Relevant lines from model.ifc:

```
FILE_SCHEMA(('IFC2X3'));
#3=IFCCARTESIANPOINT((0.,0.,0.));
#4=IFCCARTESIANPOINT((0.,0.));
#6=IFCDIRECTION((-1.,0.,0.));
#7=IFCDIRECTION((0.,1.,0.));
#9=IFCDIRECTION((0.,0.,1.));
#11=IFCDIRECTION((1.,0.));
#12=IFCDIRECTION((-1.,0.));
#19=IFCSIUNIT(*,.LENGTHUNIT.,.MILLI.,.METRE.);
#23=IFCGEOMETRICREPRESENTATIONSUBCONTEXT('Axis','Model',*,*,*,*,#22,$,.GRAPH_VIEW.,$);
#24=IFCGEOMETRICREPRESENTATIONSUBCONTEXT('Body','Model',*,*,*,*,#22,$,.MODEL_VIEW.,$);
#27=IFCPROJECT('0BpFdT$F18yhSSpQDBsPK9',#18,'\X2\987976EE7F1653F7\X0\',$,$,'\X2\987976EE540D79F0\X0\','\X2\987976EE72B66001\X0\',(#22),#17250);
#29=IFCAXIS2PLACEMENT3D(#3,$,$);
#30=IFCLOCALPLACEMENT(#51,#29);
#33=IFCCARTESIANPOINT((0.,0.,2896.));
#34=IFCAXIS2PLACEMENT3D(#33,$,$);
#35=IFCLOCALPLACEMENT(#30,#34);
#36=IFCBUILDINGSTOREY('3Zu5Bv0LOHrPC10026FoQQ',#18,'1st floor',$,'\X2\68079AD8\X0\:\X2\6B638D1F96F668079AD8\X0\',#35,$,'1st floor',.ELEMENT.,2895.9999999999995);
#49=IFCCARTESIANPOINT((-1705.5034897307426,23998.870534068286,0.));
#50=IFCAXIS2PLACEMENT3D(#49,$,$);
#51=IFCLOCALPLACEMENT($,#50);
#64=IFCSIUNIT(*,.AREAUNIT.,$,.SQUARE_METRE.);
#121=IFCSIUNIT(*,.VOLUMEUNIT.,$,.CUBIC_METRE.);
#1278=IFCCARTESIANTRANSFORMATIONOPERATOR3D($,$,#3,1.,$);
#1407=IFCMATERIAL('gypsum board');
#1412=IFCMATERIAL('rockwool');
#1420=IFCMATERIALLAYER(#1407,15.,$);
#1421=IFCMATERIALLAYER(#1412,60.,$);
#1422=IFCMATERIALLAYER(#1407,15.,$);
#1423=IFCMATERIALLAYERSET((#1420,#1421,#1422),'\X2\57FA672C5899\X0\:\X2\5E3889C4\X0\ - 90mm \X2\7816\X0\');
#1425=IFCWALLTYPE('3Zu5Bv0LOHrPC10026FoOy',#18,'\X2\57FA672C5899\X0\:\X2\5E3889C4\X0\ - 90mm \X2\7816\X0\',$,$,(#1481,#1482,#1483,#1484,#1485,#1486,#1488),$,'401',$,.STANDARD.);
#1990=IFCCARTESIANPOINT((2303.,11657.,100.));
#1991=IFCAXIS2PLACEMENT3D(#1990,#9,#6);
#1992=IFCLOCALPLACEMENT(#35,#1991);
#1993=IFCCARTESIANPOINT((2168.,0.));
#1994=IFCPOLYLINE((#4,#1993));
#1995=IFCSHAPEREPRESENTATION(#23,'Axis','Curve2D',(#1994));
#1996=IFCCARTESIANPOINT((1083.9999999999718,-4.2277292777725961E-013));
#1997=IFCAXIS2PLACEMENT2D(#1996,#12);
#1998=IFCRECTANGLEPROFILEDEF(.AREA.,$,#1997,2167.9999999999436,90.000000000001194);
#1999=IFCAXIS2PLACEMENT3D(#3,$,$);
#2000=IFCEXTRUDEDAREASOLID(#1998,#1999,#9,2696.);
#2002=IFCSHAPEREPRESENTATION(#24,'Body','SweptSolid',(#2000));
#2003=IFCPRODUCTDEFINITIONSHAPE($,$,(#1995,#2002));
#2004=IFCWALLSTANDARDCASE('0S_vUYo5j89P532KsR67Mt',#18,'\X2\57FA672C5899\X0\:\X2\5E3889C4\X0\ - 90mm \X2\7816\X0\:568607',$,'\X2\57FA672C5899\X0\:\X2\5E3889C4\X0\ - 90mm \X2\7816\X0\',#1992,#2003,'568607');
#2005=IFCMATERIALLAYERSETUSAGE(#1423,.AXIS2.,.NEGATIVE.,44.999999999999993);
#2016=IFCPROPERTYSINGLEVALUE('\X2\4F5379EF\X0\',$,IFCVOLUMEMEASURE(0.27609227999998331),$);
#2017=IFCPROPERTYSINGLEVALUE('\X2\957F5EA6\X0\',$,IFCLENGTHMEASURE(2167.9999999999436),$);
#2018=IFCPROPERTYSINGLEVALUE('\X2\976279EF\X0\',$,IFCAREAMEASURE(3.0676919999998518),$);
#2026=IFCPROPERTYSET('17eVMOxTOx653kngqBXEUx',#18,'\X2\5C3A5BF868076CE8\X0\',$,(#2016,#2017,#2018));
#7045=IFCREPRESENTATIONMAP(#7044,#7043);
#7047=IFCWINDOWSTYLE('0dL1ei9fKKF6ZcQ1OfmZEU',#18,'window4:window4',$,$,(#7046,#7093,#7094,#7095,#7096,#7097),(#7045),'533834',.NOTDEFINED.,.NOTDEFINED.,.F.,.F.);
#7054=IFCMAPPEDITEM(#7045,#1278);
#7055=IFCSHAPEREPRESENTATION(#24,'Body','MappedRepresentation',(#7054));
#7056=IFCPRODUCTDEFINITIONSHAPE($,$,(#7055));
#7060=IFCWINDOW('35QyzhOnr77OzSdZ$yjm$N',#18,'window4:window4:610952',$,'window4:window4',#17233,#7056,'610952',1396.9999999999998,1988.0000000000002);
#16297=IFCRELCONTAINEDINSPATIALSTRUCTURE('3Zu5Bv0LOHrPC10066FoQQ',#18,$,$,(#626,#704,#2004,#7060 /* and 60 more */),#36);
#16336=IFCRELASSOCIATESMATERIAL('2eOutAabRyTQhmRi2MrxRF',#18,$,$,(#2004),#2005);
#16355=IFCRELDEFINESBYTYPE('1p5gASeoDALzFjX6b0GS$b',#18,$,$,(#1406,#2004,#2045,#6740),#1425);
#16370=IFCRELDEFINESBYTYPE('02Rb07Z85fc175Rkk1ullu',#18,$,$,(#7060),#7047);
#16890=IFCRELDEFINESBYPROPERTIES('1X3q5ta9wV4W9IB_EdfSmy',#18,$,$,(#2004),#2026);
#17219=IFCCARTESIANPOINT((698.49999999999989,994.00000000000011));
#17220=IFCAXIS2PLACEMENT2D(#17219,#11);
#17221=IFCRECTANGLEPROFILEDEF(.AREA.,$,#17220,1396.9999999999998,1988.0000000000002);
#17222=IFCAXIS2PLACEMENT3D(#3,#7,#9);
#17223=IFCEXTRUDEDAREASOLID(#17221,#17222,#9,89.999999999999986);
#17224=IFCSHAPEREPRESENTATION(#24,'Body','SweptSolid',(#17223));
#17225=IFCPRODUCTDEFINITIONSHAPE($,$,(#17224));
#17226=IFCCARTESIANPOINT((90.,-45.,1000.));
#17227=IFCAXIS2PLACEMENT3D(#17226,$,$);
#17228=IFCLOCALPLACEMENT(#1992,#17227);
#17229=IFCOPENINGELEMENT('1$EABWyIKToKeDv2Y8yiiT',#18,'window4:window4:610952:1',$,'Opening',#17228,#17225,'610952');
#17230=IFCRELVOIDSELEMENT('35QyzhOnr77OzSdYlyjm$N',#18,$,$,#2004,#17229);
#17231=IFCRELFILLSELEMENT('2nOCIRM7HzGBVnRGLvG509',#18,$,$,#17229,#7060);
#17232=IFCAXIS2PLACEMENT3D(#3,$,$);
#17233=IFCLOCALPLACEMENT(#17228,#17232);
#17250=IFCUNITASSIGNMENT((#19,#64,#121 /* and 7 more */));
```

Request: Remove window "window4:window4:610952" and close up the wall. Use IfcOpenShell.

```python
import ifcopenshell
import ifcopenshell.api.feature
import ifcopenshell.api.pset
import ifcopenshell.api.root
import ifcopenshell.geom
import ifcopenshell.util.element
import ifcopenshell.util.shape
import ifcopenshell.util.unit

model = ifcopenshell.open("model.ifc")
area_scale = ifcopenshell.util.unit.calculate_unit_scale(model, "AREAUNIT")
volume_scale = ifcopenshell.util.unit.calculate_unit_scale(model, "VOLUMEUNIT")
settings = ifcopenshell.geom.settings()


def volume(element):
    """Net volume in cubic metres, openings subtracted."""
    shape = ifcopenshell.geom.create_shape(settings, element)
    return ifcopenshell.util.shape.get_volume(shape.geometry)


window = model.by_guid("35QyzhOnr77OzSdZ$yjm$N")
opening = window.FillsVoids[0].RelatingOpeningElement
wall = opening.VoidsElements[0].RelatingBuildingElement
before = volume(wall)

ifcopenshell.api.root.remove_product(model, product=window)
ifcopenshell.api.feature.remove_feature(model, feature=opening)

after = volume(wall)
thickness = 0.09  # wall thickness in metres

# Update the wall's stored quantities.
pset = model.by_id(ifcopenshell.util.element.get_pset(wall, "尺寸标注", should_inherit=False)["id"])
ifcopenshell.api.pset.edit_pset(model, pset=pset, properties={
    "体积": model.create_entity("IfcVolumeMeasure", after / volume_scale),
    "面积": model.create_entity("IfcAreaMeasure", after / thickness / area_scale),
})

print(f"wall volume {before:.3f} -> {after:.3f} m3")

model.write("model_edited.ifc")
```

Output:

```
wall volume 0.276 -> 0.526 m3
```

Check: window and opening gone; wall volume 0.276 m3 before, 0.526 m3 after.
